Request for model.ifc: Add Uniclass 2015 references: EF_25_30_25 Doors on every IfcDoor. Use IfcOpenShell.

First a look at what the model holds.

```python
import ifcopenshell

model = ifcopenshell.open("model.ifc")
print(model.schema)
print("classifications:", [c.Name for c in model.by_type("IfcClassification")])
for ifc_class in ("IfcDoor", "IfcRoof", "IfcStair", "IfcWall", "IfcWindow"):
    print(ifc_class, len(model.by_type(ifc_class)))
```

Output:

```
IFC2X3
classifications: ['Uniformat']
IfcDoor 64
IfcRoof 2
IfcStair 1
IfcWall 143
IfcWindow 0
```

```python
import ifcopenshell
import ifcopenshell.api.classification

model = ifcopenshell.open("model.ifc")

# IFC2X3 requires Source and Edition and has no link from the project to the system.
system = model.create_entity("IfcClassification", Source="NBS", Edition="2015", Name="Uniclass 2015")

codes = {
    "IfcDoor": ("EF_25_30_25", "Doors"),
}
for ifc_class, (code, name) in codes.items():
    products = model.by_type(ifc_class)
    ifcopenshell.api.classification.add_reference(
        model, products=products, classification=system, identification=code, name=name
    )
    print(code, len(products))

model.write("model_updated.ifc")
```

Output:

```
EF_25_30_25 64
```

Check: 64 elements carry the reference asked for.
